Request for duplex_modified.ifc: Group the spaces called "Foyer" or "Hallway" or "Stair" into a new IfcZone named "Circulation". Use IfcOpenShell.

First a look at what the model holds.

```python
import ifcopenshell

model = ifcopenshell.open("duplex_modified.ifc")
print(model.schema)
seen = {}
for space in model.by_type("IfcSpace"):
    seen[space.LongName] = seen.get(space.LongName, 0) + 1
for name, count in sorted(seen.items(), key=str):
    print(count, "x", name)
print("zones:", [z.Name for z in model.by_type("IfcZone")][:20])
```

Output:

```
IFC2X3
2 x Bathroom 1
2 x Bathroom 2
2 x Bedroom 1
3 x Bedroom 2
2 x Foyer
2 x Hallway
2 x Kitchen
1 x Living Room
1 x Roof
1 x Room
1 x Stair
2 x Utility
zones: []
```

```python
import ifcopenshell
import ifcopenshell.api.group
import ifcopenshell.api.root

model = ifcopenshell.open("duplex_modified.ifc")

names = {"Foyer", "Hallway", "Stair"}
spaces = [s for s in model.by_type("IfcSpace") if s.LongName in names]

zone = ifcopenshell.api.root.create_entity(model, ifc_class="IfcZone", name="Circulation")
ifcopenshell.api.group.assign_group(model, products=spaces, group=zone)
print(len(spaces), "spaces in", zone.Name)

model.write("duplex_modified_edited.ifc")
```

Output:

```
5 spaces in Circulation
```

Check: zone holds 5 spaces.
